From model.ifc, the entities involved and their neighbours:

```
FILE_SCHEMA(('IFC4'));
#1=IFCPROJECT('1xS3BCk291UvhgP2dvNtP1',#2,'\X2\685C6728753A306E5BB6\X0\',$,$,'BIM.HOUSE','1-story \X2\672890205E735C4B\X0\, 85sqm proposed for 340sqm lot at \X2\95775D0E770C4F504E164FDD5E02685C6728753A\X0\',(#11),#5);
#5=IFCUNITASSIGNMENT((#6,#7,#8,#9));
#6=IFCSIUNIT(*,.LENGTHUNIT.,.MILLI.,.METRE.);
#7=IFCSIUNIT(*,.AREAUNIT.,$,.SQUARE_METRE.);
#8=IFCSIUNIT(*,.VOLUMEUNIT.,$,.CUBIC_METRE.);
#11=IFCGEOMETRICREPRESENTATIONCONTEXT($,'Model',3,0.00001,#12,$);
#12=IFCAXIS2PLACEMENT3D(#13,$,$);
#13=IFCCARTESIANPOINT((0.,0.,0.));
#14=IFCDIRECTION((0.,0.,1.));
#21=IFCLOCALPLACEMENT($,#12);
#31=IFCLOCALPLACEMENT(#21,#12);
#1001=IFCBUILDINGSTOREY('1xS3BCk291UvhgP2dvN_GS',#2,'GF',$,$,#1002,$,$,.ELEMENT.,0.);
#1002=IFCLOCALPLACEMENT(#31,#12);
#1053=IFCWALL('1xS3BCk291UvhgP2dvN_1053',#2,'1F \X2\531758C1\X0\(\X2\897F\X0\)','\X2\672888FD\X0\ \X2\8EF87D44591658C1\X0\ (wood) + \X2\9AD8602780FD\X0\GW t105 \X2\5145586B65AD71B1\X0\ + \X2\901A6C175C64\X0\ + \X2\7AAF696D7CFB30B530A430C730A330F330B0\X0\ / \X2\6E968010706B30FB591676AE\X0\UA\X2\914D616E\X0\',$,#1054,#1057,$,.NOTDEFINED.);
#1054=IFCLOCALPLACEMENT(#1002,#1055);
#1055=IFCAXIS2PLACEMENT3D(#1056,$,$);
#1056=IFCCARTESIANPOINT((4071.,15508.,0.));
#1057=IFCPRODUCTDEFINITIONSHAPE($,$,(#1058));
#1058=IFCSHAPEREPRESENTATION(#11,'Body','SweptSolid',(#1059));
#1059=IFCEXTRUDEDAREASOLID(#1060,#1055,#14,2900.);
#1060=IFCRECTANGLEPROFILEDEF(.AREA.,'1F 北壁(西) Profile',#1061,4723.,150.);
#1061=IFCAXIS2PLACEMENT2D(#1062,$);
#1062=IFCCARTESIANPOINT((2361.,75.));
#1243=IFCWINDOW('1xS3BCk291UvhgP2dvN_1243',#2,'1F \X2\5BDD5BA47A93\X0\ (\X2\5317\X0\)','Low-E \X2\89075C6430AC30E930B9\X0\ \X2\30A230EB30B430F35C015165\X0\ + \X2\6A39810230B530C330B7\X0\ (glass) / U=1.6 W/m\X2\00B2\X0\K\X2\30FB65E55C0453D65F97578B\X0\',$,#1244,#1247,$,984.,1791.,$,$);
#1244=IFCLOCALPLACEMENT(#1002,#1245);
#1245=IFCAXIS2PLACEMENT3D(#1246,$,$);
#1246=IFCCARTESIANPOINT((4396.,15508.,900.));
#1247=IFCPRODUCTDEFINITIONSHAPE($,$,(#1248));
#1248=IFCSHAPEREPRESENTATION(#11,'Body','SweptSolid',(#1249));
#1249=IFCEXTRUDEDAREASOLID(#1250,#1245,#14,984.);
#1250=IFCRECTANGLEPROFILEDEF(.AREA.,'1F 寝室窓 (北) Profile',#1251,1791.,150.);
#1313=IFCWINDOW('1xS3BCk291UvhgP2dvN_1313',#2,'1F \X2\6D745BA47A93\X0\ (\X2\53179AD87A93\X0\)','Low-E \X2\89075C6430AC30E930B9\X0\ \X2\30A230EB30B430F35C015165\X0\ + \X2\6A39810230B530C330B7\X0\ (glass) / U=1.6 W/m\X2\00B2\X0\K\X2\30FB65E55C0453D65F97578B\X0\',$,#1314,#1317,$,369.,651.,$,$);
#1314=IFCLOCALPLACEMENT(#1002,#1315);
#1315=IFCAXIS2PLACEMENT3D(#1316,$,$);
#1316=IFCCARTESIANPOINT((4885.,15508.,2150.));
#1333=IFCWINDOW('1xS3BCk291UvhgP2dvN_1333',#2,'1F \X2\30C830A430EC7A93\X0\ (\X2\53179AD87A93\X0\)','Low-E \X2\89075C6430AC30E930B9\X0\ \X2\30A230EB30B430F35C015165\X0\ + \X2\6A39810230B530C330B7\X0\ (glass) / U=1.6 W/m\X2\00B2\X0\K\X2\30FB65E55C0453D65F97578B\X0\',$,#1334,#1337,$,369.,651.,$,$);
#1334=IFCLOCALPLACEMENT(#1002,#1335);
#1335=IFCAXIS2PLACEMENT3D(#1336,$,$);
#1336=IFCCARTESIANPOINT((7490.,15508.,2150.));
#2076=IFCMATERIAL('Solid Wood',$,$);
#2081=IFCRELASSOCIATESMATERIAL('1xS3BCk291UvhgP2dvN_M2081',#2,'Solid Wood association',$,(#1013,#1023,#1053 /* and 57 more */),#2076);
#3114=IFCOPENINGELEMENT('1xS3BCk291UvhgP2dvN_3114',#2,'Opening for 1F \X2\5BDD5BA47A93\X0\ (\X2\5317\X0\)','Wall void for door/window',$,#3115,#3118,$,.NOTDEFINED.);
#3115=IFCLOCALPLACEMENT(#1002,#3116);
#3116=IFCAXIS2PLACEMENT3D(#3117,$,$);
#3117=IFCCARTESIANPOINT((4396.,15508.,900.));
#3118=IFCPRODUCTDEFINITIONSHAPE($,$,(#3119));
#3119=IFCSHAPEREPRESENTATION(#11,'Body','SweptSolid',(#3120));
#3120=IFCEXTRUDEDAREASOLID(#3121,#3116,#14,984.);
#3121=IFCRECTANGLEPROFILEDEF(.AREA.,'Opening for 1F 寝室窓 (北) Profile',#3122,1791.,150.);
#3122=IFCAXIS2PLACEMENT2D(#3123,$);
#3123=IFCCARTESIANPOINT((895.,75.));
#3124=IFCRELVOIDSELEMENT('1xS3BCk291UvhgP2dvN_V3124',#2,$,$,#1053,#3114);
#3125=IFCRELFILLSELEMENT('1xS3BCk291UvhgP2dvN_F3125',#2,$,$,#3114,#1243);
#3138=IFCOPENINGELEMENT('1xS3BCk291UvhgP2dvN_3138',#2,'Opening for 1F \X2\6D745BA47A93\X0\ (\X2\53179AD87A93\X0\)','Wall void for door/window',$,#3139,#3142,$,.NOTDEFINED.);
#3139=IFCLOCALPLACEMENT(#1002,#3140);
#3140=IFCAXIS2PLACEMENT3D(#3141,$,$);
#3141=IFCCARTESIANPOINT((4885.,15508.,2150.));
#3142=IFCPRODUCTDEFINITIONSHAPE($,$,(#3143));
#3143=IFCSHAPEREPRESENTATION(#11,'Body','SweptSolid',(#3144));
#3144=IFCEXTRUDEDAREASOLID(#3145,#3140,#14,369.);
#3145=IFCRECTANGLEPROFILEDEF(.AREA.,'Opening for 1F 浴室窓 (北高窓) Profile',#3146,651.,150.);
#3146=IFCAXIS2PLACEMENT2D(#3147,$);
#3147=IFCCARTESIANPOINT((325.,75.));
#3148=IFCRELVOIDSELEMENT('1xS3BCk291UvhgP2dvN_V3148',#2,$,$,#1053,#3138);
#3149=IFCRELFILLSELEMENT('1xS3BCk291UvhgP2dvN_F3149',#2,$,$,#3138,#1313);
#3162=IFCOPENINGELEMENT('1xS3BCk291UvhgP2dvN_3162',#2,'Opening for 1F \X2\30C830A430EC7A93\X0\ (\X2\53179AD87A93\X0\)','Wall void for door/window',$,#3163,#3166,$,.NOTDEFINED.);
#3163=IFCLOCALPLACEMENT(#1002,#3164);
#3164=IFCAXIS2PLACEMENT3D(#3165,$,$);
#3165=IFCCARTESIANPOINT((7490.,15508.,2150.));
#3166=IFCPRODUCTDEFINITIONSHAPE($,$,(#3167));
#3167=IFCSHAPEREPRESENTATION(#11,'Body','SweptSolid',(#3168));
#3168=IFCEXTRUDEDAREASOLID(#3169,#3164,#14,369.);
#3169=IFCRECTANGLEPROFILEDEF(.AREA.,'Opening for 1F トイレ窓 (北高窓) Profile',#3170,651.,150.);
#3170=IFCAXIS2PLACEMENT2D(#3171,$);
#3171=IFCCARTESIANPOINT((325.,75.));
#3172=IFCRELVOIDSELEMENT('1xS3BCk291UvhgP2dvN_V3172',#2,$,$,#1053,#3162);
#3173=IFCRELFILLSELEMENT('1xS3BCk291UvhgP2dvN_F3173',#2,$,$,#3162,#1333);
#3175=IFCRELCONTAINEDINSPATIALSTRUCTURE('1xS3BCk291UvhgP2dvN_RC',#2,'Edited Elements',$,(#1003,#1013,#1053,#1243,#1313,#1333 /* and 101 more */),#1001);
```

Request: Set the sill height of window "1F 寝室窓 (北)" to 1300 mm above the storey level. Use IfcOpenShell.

```python
import numpy as np
import ifcopenshell
import ifcopenshell.api.geometry
import ifcopenshell.geom
import ifcopenshell.util.element
import ifcopenshell.util.placement
import ifcopenshell.util.shape
import ifcopenshell.util.unit

model = ifcopenshell.open("model.ifc")
unit_scale = ifcopenshell.util.unit.calculate_unit_scale(model)

window = model.by_guid("1xS3BCk291UvhgP2dvN_1243")
opening = window.FillsVoids[0].RelatingOpeningElement
storey = ifcopenshell.util.element.get_container(window, ifc_class="IfcBuildingStorey")
level = ifcopenshell.util.placement.get_local_placement(storey.ObjectPlacement)[2, 3]

# The opening's origin need not be at the sill, so measure its lowest point.
shape = ifcopenshell.geom.create_shape(ifcopenshell.geom.settings(), opening)
bottom = ifcopenshell.util.shape.get_shape_bottom_elevation(shape, shape.geometry) / unit_scale
dz = level + 1300.0 - bottom

shift = np.array([0.0, 0.0, dz])
# The window is not placed relative to its opening, so move both.
for product in (opening, window):
    matrix = ifcopenshell.util.placement.get_local_placement(product.ObjectPlacement)
    matrix[:3, 3] += shift
    ifcopenshell.api.geometry.edit_object_placement(model, product=product, matrix=matrix, is_si=False)

print(f"moved by {dz * unit_scale:+.3f} m")

model.write("model_v2.ifc")
```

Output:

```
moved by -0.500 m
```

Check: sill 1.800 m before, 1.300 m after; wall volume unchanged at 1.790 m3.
